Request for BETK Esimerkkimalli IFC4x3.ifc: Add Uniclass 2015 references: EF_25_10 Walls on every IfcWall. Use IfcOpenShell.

First a look at what the model holds.

```python
import ifcopenshell

model = ifcopenshell.open("BETK Esimerkkimalli IFC4x3.ifc")
print(model.schema)
print("classifications:", [c.Name for c in model.by_type("IfcClassification")])
for ifc_class in ("IfcDoor", "IfcRoof", "IfcStair", "IfcWall", "IfcWindow"):
    print(ifc_class, len(model.by_type(ifc_class)))
```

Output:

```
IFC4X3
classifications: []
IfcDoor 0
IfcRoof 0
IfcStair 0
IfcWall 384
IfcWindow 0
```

```python
import ifcopenshell
import ifcopenshell.api.classification

model = ifcopenshell.open("BETK Esimerkkimalli IFC4x3.ifc")

system = ifcopenshell.api.classification.add_classification(model, classification="Uniclass 2015")

codes = {
    "IfcWall": ("EF_25_10", "Walls"),
}
for ifc_class, (code, name) in codes.items():
    products = model.by_type(ifc_class)
    ifcopenshell.api.classification.add_reference(
        model, products=products, classification=system, identification=code, name=name
    )
    print(code, len(products))

model.write("BETK Esimerkkimalli IFC4x3_v2.ifc")
```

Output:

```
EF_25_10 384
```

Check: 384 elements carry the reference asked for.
